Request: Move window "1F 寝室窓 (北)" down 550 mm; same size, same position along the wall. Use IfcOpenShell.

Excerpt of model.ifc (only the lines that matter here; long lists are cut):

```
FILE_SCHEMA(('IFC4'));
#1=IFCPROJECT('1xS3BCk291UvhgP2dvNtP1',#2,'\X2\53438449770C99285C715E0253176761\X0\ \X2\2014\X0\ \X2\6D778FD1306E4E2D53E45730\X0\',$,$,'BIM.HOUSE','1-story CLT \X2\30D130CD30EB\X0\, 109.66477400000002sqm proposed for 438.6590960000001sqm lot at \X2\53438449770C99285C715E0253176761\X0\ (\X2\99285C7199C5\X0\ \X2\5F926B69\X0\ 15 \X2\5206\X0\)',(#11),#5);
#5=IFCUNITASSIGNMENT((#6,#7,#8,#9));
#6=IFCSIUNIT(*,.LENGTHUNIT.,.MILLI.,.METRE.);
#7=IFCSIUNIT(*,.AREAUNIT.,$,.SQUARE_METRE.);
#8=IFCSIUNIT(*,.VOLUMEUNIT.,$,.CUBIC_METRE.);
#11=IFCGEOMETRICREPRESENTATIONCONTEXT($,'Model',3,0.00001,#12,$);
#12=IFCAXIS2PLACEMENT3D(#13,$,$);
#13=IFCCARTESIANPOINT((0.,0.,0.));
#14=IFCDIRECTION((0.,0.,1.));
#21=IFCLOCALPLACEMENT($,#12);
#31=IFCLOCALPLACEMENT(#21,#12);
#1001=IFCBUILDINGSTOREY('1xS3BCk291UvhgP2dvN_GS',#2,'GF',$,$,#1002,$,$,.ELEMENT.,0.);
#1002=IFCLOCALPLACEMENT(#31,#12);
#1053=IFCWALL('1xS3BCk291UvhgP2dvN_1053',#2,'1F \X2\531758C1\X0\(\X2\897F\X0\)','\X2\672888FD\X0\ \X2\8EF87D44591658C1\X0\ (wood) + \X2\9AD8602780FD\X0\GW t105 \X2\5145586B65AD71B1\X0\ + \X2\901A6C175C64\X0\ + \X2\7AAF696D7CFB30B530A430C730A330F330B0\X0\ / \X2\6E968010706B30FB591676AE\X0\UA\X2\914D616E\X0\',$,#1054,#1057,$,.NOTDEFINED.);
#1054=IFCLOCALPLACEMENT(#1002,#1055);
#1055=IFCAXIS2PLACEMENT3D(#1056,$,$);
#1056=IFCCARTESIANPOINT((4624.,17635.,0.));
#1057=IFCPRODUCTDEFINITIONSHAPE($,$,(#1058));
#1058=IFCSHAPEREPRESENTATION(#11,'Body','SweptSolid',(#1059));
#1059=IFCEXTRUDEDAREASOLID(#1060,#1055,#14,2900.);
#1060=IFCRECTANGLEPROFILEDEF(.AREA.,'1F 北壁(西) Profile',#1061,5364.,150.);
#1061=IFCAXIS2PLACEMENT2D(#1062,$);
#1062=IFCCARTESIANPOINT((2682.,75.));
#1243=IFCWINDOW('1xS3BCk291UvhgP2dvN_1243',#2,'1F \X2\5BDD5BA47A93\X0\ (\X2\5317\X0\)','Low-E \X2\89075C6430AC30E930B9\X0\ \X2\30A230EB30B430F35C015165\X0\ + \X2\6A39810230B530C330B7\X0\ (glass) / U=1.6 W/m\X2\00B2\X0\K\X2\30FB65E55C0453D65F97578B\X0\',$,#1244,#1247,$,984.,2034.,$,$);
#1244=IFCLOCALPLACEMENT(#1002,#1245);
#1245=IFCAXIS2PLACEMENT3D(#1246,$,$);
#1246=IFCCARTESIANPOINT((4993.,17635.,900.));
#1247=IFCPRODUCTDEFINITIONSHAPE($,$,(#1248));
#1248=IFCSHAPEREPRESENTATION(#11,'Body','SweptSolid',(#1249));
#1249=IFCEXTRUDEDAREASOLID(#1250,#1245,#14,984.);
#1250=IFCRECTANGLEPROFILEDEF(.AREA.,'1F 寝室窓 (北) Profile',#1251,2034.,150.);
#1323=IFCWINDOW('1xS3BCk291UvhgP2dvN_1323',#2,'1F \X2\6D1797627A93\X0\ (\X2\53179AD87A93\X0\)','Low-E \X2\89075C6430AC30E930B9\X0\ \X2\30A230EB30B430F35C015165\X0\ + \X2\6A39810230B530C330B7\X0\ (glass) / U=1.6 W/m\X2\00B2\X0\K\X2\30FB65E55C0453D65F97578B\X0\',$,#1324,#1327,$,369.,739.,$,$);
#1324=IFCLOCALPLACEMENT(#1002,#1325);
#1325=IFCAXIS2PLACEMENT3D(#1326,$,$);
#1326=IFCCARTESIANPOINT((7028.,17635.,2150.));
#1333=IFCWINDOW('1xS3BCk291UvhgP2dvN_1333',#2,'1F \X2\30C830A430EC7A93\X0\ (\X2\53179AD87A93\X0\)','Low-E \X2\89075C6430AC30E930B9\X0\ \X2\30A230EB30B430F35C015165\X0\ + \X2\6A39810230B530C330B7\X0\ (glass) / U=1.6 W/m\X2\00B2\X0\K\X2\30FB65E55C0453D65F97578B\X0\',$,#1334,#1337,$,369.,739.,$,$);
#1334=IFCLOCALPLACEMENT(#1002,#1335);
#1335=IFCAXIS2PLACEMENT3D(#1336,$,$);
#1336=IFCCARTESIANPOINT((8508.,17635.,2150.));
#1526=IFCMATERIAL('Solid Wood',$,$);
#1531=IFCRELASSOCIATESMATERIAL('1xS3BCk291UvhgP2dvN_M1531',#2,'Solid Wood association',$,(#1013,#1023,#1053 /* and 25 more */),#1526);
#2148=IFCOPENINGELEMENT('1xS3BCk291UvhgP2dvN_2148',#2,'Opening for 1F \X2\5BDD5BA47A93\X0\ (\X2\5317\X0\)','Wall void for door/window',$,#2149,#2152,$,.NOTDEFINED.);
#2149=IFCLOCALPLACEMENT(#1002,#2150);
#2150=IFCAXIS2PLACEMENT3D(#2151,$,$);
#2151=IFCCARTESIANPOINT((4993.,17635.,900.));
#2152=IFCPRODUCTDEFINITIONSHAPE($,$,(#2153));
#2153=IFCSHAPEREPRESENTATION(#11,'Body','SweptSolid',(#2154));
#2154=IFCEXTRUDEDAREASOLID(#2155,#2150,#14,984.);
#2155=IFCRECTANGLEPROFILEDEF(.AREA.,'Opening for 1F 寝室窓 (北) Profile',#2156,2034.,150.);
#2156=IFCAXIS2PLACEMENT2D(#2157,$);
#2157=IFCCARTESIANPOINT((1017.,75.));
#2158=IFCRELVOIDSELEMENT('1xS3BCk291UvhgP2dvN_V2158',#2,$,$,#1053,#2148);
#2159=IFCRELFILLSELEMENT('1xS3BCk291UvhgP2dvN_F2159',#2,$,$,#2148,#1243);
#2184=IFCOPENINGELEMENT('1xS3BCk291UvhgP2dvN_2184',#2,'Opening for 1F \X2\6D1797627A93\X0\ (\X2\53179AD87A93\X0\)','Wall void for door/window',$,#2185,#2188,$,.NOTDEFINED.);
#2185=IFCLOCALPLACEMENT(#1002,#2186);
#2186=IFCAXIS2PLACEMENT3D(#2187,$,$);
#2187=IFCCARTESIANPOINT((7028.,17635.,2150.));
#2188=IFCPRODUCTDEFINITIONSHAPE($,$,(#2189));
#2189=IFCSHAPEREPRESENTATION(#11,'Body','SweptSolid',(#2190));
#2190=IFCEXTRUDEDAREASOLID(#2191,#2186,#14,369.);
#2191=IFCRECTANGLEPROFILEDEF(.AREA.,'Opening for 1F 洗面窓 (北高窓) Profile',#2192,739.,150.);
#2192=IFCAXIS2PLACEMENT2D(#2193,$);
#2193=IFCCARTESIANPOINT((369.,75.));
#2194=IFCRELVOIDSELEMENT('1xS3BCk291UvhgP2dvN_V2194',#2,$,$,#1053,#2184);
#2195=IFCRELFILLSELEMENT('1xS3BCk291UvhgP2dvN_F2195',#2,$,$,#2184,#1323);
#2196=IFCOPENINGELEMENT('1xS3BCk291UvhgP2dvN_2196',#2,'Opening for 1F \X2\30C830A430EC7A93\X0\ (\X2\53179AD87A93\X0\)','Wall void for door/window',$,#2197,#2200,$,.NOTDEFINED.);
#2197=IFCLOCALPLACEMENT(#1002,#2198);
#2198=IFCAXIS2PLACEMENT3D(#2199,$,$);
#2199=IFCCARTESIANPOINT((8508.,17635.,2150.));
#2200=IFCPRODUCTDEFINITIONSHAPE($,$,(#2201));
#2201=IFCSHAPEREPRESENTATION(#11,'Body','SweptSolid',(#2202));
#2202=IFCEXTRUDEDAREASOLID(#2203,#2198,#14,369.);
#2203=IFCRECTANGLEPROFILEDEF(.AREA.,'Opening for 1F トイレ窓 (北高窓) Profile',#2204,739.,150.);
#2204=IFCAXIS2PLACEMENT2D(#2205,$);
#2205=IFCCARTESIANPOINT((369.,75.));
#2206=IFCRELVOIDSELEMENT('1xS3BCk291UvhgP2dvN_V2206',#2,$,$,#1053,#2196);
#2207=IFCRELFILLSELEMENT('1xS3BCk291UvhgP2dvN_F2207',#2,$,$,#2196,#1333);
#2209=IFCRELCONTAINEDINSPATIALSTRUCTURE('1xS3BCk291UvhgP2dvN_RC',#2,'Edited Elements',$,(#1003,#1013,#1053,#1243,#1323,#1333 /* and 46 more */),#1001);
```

```python
import numpy as np
import ifcopenshell
import ifcopenshell.api.geometry
import ifcopenshell.util.placement
import ifcopenshell.util.unit

model = ifcopenshell.open("model.ifc")
unit_scale = ifcopenshell.util.unit.calculate_unit_scale(model)

window = model.by_id(1243)
opening = window.FillsVoids[0].RelatingOpeningElement
dz = -0.55 / unit_scale

shift = np.array([0.0, 0.0, dz])
# The window is not placed relative to its opening, so move both.
for product in (opening, window):
    matrix = ifcopenshell.util.placement.get_local_placement(product.ObjectPlacement)
    matrix[:3, 3] += shift
    ifcopenshell.api.geometry.edit_object_placement(model, product=product, matrix=matrix, is_si=False)

print(f"moved by {dz * unit_scale:+.3f} m")

model.write("model_rev.ifc")
```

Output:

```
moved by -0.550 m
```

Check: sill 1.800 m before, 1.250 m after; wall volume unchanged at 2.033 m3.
